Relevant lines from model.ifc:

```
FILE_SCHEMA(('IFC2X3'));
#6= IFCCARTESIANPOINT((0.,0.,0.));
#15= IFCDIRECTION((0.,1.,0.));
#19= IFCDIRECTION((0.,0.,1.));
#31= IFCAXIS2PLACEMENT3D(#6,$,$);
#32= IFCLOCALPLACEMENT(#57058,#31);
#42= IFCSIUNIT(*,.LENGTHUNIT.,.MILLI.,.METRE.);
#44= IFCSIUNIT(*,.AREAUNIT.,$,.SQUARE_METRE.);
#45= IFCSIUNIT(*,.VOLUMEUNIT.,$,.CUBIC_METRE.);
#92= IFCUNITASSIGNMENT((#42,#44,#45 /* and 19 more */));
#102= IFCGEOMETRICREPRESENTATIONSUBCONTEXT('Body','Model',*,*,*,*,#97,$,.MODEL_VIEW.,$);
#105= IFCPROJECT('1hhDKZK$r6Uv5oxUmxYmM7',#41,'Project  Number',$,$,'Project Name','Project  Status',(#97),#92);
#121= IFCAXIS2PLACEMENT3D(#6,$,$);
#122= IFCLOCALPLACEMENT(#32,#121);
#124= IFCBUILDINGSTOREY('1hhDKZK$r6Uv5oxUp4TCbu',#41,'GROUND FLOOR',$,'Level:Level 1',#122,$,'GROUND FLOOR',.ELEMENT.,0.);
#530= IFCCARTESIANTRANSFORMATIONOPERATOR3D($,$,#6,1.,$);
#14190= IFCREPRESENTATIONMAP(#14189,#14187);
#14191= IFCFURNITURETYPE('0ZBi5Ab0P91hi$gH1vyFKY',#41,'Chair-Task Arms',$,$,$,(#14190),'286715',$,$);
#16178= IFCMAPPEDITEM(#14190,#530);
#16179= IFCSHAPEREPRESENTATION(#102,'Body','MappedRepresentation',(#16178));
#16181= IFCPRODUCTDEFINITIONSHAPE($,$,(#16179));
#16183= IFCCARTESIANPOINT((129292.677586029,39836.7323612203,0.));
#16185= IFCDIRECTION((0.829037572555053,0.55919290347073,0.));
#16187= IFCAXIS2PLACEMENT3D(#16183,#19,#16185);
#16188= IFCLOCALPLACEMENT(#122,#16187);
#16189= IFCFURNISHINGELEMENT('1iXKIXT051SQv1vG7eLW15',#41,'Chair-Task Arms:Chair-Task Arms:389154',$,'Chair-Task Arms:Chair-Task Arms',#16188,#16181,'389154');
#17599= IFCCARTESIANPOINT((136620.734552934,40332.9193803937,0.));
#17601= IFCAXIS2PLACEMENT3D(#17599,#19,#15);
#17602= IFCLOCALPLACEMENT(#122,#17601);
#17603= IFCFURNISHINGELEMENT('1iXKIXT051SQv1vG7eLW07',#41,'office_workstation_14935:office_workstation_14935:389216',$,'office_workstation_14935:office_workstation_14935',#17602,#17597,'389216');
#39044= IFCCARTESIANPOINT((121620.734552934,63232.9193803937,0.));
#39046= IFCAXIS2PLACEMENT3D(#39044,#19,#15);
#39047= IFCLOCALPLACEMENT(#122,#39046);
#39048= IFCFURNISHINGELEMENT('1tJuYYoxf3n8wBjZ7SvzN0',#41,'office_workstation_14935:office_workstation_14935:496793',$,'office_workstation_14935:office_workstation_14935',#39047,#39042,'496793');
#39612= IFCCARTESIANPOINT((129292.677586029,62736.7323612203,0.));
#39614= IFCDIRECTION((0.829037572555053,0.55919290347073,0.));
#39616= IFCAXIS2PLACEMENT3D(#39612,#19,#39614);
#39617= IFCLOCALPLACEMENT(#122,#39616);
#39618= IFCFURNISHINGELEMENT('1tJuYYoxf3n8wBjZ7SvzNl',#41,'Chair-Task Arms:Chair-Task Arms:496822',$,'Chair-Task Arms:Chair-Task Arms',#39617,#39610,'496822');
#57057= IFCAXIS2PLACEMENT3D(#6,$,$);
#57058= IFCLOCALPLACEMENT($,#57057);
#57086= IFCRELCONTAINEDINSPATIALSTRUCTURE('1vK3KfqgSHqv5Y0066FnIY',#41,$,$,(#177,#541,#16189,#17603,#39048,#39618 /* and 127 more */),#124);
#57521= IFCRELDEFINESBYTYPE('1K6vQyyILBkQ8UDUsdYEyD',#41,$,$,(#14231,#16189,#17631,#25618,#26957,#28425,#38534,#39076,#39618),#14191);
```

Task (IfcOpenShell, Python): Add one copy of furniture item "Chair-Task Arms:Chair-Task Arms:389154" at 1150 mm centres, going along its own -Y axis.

```python
import ifcopenshell
import ifcopenshell.api.geometry
import ifcopenshell.api.root
import ifcopenshell.util.element
import ifcopenshell.util.placement
import ifcopenshell.util.unit

model = ifcopenshell.open("model.ifc")
unit_scale = ifcopenshell.util.unit.calculate_unit_scale(model)


def reuse_history(source, copy):
    """copy_class also copies each property set's owner history, people and application; keep the originals."""
    for rel in copy.IsDefinedBy:
        if rel.is_a("IfcRelDefinesByProperties") and (history := rel.RelatingPropertyDefinition.OwnerHistory):
            rel.RelatingPropertyDefinition.OwnerHistory = source.OwnerHistory
            ifcopenshell.util.element.remove_deep2(model, history)


source = model.by_guid("1iXKIXT051SQv1vG7eLW15")
base = ifcopenshell.util.placement.get_local_placement(source.ObjectPlacement)
step = -base[:3, 1] * 1.15 / unit_scale

for i in range(1, 2):
    copy = ifcopenshell.api.root.copy_class(model, product=source)
    copy.Representation = ifcopenshell.util.element.copy_deep(
        model, source.Representation, exclude=["IfcGeometricRepresentationContext", "IfcRepresentationMap"]
    )
    copy.Name = "Chair-Task Arms:Chair-Task Arms"
    copy.Tag = None
    reuse_history(source, copy)
    matrix = base.copy()
    matrix[:3, 3] += i * step
    print("added at", matrix[:3, 3].round(3) + 0.0)
    ifcopenshell.api.geometry.edit_object_placement(model, product=copy, matrix=matrix, is_si=False)

model.write("model_edited.ifc")
```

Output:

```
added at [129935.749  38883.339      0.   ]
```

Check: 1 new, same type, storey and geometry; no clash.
